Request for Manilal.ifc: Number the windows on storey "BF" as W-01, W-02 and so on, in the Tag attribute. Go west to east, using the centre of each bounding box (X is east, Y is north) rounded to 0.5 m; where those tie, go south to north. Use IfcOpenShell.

First a look at what the model holds.

```python
import ifcopenshell
import ifcopenshell.util.element
import ifcopenshell.util.placement

model = ifcopenshell.open("Manilal.ifc")
print(model.schema)
storey = next(s for s in model.by_type("IfcBuildingStorey") if s.Name == "BF")
windows = [e for e in ifcopenshell.util.element.get_decomposition(storey) if e.is_a("IfcWindow")]
for e in sorted(windows, key=lambda e: e.id()):
    origin = ifcopenshell.util.placement.get_local_placement(e.ObjectPlacement)[:3, 3]
    print(e.id(), e.Tag, e.Name, origin.round(2) + 0.0, sep=" | ")
```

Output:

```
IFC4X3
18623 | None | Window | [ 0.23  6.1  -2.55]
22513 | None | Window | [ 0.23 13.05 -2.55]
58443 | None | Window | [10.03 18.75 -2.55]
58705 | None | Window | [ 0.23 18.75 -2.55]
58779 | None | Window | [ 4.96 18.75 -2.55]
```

```python
import ifcopenshell
import ifcopenshell.geom
import ifcopenshell.util.element
import ifcopenshell.util.shape

model = ifcopenshell.open("Manilal.ifc")
settings = ifcopenshell.geom.settings()
settings.set("use-world-coords", True)


def centre(element):
    shape = ifcopenshell.geom.create_shape(settings, element)
    return ifcopenshell.util.shape.get_bbox_centroid(shape.geometry)


storey = next(s for s in model.by_type("IfcBuildingStorey") if s.Name == "BF")
windows = [e for e in ifcopenshell.util.element.get_decomposition(storey) if e.is_a("IfcWindow")]

# Insertion points can sit at a corner or the storey origin, so sort by the geometry (in metres).
centres = {e: centre(e) for e in windows}
windows.sort(key=lambda e: (round(centres[e][0] / 0.5), centres[e][1]))

for i, e in enumerate(windows, start=1):
    number = f"W-{i:02d}"
    e.Tag = number
    print(e.id(), number)

model.write("Manilal_edited.ifc")
```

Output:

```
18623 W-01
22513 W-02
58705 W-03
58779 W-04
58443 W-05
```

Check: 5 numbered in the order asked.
